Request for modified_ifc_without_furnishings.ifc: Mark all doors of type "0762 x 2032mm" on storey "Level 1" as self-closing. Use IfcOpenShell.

First a look at what the model holds.

```python
import ifcopenshell
import ifcopenshell.util.element

model = ifcopenshell.open("modified_ifc_without_furnishings.ifc")
print(model.schema)
storey = next(s for s in model.by_type("IfcBuildingStorey") if s.Name == "Level 1")
doors = [e for e in ifcopenshell.util.element.get_decomposition(storey) if e.is_a("IfcDoor")]
seen = {}
for e in doors:
    element_type = ifcopenshell.util.element.get_type(e)
    key = (element_type.Name if element_type != e and element_type else None, ifcopenshell.util.element.get_pset(e, "Pset_DoorCommon", "SelfClosing"))
    seen[key] = seen.get(key, 0) + 1
for (name, value), count in sorted(seen.items(), key=str):
    print(count, "x", name, "|", value)
```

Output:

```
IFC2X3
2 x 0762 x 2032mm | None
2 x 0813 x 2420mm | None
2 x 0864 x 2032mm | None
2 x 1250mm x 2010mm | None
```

```python
import ifcopenshell
import ifcopenshell.api.pset
import ifcopenshell.util.element

model = ifcopenshell.open("modified_ifc_without_furnishings.ifc")

storey = next(s for s in model.by_type("IfcBuildingStorey") if s.Name == "Level 1")
doors = [e for e in ifcopenshell.util.element.get_decomposition(storey) if e.is_a("IfcDoor")]

count = 0
for e in doors:
    element_type = ifcopenshell.util.element.get_type(e)
    if element_type in (None, e) or element_type.Name != "0762 x 2032mm":
        continue
    # add_pset returns the element's existing set when there is one.
    pset = ifcopenshell.api.pset.add_pset(model, product=e, name="Pset_DoorCommon")
    ifcopenshell.api.pset.edit_pset(model, pset=pset, properties={"SelfClosing": True})
    count += 1

print(count, "doors updated")

model.write("modified_ifc_without_furnishings_edited.ifc")
```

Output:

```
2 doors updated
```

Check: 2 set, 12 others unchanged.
